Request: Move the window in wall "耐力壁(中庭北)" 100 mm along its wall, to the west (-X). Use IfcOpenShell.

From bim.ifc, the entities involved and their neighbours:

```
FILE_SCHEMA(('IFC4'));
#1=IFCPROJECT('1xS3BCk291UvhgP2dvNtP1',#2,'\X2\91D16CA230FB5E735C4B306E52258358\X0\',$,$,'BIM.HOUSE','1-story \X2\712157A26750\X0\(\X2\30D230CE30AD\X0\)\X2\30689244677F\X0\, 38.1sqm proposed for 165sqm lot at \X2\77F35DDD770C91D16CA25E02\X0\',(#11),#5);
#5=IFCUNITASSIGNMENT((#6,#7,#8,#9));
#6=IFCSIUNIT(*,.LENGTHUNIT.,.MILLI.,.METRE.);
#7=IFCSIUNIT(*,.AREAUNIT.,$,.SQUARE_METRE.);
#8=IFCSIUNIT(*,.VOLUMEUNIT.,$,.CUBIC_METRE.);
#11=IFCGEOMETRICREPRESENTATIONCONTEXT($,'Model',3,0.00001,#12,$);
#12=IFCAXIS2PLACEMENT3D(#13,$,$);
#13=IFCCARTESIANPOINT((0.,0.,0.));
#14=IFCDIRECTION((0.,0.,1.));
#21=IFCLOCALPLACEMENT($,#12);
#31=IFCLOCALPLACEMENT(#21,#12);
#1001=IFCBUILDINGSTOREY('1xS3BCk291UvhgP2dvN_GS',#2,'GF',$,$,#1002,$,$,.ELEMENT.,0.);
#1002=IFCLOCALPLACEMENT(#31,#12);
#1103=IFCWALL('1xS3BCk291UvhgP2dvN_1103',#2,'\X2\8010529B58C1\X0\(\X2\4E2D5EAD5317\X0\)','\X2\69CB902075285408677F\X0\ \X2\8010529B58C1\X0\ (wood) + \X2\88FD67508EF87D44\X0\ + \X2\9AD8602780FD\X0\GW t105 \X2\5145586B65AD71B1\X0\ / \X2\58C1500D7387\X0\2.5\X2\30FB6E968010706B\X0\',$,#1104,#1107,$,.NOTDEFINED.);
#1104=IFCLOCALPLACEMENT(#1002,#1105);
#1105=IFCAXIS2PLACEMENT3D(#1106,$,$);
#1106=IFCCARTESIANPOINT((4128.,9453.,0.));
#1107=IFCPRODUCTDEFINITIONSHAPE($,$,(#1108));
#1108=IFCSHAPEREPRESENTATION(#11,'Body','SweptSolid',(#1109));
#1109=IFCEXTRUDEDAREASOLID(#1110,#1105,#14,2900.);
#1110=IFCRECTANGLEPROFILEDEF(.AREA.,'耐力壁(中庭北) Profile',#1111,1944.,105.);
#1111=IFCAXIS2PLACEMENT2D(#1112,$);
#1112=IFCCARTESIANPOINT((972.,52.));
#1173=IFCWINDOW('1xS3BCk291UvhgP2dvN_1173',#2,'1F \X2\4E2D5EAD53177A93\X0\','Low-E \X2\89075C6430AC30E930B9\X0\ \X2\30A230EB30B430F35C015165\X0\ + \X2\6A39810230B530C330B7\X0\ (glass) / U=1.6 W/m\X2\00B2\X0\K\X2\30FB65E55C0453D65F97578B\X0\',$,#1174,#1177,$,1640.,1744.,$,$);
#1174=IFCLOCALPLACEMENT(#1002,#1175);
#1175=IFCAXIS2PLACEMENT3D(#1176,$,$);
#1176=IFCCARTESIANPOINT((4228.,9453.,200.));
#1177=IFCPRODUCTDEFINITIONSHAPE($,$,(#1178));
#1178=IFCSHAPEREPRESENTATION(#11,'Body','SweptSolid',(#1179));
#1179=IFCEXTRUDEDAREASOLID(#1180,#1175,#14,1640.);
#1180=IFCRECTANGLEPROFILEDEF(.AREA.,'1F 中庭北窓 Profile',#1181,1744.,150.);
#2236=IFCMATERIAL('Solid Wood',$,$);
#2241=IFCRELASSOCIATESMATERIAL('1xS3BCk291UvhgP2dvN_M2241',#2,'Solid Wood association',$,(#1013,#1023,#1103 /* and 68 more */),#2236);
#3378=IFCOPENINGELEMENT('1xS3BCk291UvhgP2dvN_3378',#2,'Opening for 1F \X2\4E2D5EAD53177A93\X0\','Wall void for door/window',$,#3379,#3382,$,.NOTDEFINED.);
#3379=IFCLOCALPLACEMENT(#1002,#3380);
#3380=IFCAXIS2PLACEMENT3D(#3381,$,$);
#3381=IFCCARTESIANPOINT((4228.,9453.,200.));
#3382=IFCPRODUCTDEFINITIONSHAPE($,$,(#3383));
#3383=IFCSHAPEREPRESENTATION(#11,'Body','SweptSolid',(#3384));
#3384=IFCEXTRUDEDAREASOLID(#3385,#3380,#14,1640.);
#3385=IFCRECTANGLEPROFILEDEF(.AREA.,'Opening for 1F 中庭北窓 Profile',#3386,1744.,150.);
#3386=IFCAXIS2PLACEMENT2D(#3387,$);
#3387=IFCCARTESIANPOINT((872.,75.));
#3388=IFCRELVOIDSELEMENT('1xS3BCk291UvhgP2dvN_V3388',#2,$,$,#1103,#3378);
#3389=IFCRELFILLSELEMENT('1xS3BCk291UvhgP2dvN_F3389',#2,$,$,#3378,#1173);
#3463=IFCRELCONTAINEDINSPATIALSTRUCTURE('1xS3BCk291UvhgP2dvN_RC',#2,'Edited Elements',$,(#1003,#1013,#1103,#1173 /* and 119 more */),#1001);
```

```python
import ifcopenshell
import ifcopenshell.api.geometry
import ifcopenshell.util.placement

model = ifcopenshell.open("bim.ifc")

window = model.by_guid("1xS3BCk291UvhgP2dvN_1173")
opening = window.FillsVoids[0].RelatingOpeningElement
wall = opening.VoidsElements[0].RelatingBuildingElement

wall_matrix = ifcopenshell.util.placement.get_local_placement(wall.ObjectPlacement)
shift = wall_matrix[:3, 0] * -100.0
before = ifcopenshell.util.placement.get_local_placement(window.ObjectPlacement)[:3, 3].copy()

# The window is not placed relative to its opening, so move both.
for product in (opening, window):
    matrix = ifcopenshell.util.placement.get_local_placement(product.ObjectPlacement)
    matrix[:3, 3] += shift
    ifcopenshell.api.geometry.edit_object_placement(model, product=product, matrix=matrix, is_si=False)

after = ifcopenshell.util.placement.get_local_placement(window.ObjectPlacement)[:3, 3]
print("window moved by", (after - before).round(3) + 0.0)

model.write("bim_rev.ifc")
```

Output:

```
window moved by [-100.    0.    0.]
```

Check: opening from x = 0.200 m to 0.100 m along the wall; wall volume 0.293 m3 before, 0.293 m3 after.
